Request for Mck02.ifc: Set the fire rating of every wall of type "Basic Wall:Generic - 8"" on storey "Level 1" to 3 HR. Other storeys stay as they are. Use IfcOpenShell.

First a look at what the model holds.

```python
import ifcopenshell
import ifcopenshell.util.element

model = ifcopenshell.open("Mck02.ifc")
print(model.schema)
storey = next(s for s in model.by_type("IfcBuildingStorey") if s.Name == "Level 1")
walls = [e for e in ifcopenshell.util.element.get_decomposition(storey) if e.is_a("IfcWall")]
seen = {}
for e in walls:
    element_type = ifcopenshell.util.element.get_type(e)
    key = (element_type.Name if element_type != e and element_type else None, ifcopenshell.util.element.get_pset(e, "Pset_WallCommon", "FireRating"))
    seen[key] = seen.get(key, 0) + 1
for (name, value), count in sorted(seen.items(), key=str):
    print(count, "x", name, "|", value)
```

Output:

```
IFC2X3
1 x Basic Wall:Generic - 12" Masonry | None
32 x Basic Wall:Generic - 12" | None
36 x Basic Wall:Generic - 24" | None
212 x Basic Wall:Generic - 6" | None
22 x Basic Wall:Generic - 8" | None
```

```python
import ifcopenshell
import ifcopenshell.api.pset
import ifcopenshell.util.element

model = ifcopenshell.open("Mck02.ifc")

storey = next(s for s in model.by_type("IfcBuildingStorey") if s.Name == "Level 1")
walls = [e for e in ifcopenshell.util.element.get_decomposition(storey) if e.is_a("IfcWall")]

count = 0
for e in walls:
    element_type = ifcopenshell.util.element.get_type(e)
    if element_type in (None, e) or element_type.Name != 'Basic Wall:Generic - 8"':
        continue
    # add_pset returns the element's existing set when there is one.
    pset = ifcopenshell.api.pset.add_pset(model, product=e, name="Pset_WallCommon")
    ifcopenshell.api.pset.edit_pset(model, pset=pset, properties={"FireRating": "3 HR"})
    count += 1

print(count, "walls updated")

model.write("Mck02_edited.ifc")
```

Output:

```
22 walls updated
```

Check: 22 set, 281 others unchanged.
